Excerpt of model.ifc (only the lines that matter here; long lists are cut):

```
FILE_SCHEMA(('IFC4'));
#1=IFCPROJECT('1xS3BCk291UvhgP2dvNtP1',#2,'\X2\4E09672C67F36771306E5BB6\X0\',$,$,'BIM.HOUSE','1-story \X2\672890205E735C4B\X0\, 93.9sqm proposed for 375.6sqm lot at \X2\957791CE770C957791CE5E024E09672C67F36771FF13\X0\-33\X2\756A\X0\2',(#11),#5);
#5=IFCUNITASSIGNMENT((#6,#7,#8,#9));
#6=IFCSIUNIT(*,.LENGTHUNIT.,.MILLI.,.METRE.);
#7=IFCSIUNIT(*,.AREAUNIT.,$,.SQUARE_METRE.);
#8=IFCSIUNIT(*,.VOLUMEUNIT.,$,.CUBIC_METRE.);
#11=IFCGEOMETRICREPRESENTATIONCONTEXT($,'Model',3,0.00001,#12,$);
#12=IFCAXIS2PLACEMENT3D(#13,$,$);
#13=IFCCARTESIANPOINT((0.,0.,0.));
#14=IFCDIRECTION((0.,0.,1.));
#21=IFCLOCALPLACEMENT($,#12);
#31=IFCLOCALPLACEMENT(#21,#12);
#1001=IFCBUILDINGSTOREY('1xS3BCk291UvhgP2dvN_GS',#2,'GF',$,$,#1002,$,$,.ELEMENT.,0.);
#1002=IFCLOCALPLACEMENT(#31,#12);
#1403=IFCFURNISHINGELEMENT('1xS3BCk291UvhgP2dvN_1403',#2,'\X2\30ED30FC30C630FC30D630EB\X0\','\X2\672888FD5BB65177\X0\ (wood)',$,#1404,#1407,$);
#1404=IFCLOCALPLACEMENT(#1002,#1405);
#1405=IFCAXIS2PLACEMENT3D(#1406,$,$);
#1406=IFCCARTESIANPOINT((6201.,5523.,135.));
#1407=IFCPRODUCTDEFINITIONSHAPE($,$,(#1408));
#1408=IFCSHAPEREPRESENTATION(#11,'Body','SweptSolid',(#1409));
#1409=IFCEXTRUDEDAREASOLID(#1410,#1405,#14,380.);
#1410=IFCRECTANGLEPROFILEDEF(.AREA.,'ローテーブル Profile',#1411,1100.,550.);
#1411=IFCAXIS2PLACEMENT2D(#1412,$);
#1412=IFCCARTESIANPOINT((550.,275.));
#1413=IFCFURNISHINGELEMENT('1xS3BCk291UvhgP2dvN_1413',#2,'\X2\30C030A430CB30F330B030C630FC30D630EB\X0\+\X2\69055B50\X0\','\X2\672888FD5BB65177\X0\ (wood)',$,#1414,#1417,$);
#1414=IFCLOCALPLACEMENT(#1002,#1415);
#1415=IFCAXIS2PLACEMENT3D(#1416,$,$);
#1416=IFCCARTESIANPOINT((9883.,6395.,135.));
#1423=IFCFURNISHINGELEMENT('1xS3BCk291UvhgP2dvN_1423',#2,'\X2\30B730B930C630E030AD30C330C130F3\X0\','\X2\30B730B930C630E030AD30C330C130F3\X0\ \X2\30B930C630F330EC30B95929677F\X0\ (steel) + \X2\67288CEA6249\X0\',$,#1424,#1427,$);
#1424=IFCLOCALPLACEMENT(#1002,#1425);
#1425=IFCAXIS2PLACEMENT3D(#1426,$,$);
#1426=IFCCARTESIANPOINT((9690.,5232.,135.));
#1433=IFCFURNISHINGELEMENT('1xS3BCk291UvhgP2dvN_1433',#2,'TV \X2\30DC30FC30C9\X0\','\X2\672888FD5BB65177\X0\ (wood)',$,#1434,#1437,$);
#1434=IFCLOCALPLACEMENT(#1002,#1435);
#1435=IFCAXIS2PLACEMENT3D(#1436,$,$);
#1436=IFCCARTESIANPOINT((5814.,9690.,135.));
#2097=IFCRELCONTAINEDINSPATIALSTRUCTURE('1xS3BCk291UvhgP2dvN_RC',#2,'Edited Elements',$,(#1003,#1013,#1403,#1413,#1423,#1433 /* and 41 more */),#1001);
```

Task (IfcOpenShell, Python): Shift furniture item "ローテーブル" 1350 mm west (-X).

```python
import ifcopenshell
import ifcopenshell.api.geometry
import ifcopenshell.util.placement

model = ifcopenshell.open("model.ifc")

item = model.by_id(1403)
matrix = ifcopenshell.util.placement.get_local_placement(item.ObjectPlacement)
matrix[0, 3] -= 1350.0
ifcopenshell.api.geometry.edit_object_placement(model, product=item, matrix=matrix, is_si=False)

print(ifcopenshell.util.placement.get_local_placement(item.ObjectPlacement).round(3) + 0.0)

model.write("model-out.ifc")
```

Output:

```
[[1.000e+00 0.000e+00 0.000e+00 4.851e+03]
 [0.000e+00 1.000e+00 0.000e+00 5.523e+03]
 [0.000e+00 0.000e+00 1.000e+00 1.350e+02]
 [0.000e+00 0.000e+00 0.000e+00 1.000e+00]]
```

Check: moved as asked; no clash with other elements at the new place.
